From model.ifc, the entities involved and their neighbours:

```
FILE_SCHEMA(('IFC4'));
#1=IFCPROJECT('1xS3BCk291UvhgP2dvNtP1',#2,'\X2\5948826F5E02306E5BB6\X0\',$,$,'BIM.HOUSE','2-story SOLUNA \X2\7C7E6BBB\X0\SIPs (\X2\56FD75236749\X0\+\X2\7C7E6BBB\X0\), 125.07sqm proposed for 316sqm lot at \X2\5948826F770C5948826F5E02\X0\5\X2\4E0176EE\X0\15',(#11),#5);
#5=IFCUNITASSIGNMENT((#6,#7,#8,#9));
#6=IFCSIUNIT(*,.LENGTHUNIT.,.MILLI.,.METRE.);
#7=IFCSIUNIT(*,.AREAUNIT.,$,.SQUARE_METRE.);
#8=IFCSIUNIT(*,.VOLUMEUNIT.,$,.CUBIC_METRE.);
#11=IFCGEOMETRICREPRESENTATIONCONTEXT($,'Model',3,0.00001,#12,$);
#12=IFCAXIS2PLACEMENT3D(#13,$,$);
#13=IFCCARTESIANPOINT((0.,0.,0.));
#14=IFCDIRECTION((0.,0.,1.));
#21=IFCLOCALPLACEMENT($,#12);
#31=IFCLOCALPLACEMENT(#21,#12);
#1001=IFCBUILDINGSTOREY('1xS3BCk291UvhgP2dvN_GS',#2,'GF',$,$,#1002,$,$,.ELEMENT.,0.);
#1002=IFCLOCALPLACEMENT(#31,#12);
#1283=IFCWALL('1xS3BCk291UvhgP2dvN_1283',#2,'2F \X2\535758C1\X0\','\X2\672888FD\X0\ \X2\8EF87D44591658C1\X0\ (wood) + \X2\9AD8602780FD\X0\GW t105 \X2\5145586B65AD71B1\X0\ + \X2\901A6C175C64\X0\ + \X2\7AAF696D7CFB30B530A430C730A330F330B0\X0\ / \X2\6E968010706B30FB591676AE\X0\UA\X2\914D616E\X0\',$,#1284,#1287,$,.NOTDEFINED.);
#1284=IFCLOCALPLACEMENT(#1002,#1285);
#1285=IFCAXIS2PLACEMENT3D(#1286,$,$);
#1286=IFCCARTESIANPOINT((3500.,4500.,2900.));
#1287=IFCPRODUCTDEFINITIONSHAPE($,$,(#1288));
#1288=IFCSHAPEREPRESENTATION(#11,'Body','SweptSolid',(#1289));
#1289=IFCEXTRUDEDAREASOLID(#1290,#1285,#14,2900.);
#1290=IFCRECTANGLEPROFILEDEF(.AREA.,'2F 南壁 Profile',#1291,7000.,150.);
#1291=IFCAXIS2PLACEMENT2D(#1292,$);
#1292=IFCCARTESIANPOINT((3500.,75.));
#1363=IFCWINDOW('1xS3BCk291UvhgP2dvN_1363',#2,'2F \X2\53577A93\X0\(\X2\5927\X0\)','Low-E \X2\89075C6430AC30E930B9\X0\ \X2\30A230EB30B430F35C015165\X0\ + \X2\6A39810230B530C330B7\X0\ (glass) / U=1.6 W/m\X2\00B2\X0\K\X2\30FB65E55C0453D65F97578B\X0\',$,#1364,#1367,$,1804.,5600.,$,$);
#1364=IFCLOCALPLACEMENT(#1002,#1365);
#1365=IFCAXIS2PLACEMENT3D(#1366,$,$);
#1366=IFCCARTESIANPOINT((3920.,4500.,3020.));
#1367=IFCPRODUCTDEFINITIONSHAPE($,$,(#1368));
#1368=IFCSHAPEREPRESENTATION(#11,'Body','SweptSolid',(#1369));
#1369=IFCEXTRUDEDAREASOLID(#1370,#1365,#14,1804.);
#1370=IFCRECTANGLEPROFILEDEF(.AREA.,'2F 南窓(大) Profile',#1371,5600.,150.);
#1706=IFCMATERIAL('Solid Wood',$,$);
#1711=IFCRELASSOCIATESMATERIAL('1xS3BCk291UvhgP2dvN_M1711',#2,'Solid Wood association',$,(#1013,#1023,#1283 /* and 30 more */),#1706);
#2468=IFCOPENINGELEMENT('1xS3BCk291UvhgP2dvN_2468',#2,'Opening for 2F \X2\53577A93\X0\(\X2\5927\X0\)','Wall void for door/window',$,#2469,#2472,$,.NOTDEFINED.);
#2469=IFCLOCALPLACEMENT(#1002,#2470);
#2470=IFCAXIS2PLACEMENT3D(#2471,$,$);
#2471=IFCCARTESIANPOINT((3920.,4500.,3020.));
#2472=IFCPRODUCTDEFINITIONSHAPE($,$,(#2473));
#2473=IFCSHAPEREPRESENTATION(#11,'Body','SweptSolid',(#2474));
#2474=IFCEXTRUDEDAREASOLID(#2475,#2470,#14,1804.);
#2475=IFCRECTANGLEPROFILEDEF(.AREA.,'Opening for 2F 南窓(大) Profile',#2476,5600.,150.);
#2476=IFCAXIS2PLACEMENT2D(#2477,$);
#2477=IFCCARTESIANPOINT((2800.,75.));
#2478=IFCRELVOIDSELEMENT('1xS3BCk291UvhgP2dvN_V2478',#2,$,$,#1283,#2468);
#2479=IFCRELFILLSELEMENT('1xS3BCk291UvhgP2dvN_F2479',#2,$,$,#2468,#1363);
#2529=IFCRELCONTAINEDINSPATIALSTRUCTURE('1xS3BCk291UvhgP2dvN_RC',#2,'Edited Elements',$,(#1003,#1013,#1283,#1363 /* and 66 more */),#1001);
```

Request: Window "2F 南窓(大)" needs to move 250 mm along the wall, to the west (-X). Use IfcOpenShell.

```python
import ifcopenshell
import ifcopenshell.api.geometry
import ifcopenshell.util.placement
import ifcopenshell.util.unit

model = ifcopenshell.open("model.ifc")
unit_scale = ifcopenshell.util.unit.calculate_unit_scale(model)

window = model.by_guid("1xS3BCk291UvhgP2dvN_1363")
opening = window.FillsVoids[0].RelatingOpeningElement
wall = opening.VoidsElements[0].RelatingBuildingElement

wall_matrix = ifcopenshell.util.placement.get_local_placement(wall.ObjectPlacement)
shift = wall_matrix[:3, 0] * -0.25 / unit_scale
before = ifcopenshell.util.placement.get_local_placement(window.ObjectPlacement)[:3, 3].copy()

# The window is not placed relative to its opening, so move both.
for product in (opening, window):
    matrix = ifcopenshell.util.placement.get_local_placement(product.ObjectPlacement)
    matrix[:3, 3] += shift
    ifcopenshell.api.geometry.edit_object_placement(model, product=product, matrix=matrix, is_si=False)

after = ifcopenshell.util.placement.get_local_placement(window.ObjectPlacement)[:3, 3]
print("window moved by", (after - before).round(3) + 0.0)

model.write("model-out.ifc")
```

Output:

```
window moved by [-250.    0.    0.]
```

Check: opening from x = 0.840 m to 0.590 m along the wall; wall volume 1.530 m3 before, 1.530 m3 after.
